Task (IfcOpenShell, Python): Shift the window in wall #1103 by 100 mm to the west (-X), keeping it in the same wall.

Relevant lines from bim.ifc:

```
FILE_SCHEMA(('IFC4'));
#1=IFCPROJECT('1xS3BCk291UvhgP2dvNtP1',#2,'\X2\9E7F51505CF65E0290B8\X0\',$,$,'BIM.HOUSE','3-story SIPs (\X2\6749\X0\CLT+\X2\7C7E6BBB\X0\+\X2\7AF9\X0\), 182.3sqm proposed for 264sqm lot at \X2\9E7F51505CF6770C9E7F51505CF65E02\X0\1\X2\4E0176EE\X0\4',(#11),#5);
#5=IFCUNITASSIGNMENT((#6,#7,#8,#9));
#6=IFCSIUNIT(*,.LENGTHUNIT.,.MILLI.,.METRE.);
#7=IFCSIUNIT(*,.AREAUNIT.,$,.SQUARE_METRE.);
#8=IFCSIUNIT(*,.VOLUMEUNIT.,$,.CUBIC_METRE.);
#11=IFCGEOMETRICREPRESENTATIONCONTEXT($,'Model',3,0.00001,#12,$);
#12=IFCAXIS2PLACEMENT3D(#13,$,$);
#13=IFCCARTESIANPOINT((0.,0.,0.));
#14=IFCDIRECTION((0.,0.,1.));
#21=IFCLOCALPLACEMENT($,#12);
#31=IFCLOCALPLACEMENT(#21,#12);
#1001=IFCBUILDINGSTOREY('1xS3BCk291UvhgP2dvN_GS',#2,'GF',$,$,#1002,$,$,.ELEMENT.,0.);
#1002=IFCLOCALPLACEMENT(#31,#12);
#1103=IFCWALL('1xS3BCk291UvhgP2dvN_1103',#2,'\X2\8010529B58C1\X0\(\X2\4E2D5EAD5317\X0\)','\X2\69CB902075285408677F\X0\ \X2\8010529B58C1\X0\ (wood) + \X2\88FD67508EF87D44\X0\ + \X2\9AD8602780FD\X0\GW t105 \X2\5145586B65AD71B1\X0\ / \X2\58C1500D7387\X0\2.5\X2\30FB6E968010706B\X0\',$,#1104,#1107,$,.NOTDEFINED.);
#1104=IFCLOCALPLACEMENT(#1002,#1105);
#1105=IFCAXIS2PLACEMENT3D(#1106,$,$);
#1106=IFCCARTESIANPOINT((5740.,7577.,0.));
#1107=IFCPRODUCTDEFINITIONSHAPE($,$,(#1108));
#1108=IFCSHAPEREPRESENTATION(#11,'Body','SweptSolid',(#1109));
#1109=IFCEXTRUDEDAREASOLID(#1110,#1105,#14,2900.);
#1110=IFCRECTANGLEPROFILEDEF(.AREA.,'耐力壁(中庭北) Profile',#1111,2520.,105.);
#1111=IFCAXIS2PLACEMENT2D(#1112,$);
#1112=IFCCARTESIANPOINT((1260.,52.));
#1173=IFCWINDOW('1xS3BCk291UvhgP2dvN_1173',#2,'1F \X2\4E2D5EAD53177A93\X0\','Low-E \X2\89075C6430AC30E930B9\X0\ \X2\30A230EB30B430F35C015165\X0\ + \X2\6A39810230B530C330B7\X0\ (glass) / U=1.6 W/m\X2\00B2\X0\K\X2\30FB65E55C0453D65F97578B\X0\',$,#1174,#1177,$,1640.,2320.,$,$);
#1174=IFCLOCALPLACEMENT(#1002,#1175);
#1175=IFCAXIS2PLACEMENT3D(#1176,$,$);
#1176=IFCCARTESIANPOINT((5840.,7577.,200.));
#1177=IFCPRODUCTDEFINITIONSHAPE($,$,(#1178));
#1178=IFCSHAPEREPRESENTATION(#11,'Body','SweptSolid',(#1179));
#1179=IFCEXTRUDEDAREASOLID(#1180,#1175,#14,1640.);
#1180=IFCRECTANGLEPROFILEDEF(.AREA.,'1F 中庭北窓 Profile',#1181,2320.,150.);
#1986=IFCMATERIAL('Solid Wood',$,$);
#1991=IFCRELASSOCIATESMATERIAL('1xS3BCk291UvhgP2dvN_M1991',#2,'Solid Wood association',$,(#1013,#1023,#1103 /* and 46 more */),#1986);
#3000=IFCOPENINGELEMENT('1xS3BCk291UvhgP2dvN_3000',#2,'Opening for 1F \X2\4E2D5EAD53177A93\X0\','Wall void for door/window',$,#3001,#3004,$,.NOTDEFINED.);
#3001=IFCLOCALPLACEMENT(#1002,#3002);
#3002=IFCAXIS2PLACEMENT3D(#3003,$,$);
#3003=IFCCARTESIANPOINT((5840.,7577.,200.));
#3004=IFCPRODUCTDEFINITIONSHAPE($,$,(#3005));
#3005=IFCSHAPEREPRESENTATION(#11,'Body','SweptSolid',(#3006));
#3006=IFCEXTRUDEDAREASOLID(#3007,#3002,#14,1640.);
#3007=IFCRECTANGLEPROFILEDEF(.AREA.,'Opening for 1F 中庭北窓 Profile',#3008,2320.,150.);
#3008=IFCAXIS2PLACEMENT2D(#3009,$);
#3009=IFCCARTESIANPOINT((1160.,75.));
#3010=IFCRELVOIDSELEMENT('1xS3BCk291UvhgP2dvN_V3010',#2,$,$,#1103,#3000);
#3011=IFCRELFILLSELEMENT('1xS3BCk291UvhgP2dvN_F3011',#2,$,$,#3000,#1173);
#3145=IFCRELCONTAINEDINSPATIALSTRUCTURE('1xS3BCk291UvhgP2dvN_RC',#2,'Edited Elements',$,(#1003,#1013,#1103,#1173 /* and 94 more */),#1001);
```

```python
import ifcopenshell
import ifcopenshell.api.geometry
import ifcopenshell.util.placement
import ifcopenshell.util.unit

model = ifcopenshell.open("bim.ifc")
unit_scale = ifcopenshell.util.unit.calculate_unit_scale(model)

window = model.by_guid("1xS3BCk291UvhgP2dvN_1173")
opening = window.FillsVoids[0].RelatingOpeningElement
wall = opening.VoidsElements[0].RelatingBuildingElement

wall_matrix = ifcopenshell.util.placement.get_local_placement(wall.ObjectPlacement)
shift = wall_matrix[:3, 0] * -0.1 / unit_scale
before = ifcopenshell.util.placement.get_local_placement(window.ObjectPlacement)[:3, 3].copy()

# The window is not placed relative to its opening, so move both.
for product in (opening, window):
    matrix = ifcopenshell.util.placement.get_local_placement(product.ObjectPlacement)
    matrix[:3, 3] += shift
    ifcopenshell.api.geometry.edit_object_placement(model, product=product, matrix=matrix, is_si=False)

after = ifcopenshell.util.placement.get_local_placement(window.ObjectPlacement)[:3, 3]
print("window moved by", (after - before).round(3) + 0.0)

model.write("bim-out.ifc")
```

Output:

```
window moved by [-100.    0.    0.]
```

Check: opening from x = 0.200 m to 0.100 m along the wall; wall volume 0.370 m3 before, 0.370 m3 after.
